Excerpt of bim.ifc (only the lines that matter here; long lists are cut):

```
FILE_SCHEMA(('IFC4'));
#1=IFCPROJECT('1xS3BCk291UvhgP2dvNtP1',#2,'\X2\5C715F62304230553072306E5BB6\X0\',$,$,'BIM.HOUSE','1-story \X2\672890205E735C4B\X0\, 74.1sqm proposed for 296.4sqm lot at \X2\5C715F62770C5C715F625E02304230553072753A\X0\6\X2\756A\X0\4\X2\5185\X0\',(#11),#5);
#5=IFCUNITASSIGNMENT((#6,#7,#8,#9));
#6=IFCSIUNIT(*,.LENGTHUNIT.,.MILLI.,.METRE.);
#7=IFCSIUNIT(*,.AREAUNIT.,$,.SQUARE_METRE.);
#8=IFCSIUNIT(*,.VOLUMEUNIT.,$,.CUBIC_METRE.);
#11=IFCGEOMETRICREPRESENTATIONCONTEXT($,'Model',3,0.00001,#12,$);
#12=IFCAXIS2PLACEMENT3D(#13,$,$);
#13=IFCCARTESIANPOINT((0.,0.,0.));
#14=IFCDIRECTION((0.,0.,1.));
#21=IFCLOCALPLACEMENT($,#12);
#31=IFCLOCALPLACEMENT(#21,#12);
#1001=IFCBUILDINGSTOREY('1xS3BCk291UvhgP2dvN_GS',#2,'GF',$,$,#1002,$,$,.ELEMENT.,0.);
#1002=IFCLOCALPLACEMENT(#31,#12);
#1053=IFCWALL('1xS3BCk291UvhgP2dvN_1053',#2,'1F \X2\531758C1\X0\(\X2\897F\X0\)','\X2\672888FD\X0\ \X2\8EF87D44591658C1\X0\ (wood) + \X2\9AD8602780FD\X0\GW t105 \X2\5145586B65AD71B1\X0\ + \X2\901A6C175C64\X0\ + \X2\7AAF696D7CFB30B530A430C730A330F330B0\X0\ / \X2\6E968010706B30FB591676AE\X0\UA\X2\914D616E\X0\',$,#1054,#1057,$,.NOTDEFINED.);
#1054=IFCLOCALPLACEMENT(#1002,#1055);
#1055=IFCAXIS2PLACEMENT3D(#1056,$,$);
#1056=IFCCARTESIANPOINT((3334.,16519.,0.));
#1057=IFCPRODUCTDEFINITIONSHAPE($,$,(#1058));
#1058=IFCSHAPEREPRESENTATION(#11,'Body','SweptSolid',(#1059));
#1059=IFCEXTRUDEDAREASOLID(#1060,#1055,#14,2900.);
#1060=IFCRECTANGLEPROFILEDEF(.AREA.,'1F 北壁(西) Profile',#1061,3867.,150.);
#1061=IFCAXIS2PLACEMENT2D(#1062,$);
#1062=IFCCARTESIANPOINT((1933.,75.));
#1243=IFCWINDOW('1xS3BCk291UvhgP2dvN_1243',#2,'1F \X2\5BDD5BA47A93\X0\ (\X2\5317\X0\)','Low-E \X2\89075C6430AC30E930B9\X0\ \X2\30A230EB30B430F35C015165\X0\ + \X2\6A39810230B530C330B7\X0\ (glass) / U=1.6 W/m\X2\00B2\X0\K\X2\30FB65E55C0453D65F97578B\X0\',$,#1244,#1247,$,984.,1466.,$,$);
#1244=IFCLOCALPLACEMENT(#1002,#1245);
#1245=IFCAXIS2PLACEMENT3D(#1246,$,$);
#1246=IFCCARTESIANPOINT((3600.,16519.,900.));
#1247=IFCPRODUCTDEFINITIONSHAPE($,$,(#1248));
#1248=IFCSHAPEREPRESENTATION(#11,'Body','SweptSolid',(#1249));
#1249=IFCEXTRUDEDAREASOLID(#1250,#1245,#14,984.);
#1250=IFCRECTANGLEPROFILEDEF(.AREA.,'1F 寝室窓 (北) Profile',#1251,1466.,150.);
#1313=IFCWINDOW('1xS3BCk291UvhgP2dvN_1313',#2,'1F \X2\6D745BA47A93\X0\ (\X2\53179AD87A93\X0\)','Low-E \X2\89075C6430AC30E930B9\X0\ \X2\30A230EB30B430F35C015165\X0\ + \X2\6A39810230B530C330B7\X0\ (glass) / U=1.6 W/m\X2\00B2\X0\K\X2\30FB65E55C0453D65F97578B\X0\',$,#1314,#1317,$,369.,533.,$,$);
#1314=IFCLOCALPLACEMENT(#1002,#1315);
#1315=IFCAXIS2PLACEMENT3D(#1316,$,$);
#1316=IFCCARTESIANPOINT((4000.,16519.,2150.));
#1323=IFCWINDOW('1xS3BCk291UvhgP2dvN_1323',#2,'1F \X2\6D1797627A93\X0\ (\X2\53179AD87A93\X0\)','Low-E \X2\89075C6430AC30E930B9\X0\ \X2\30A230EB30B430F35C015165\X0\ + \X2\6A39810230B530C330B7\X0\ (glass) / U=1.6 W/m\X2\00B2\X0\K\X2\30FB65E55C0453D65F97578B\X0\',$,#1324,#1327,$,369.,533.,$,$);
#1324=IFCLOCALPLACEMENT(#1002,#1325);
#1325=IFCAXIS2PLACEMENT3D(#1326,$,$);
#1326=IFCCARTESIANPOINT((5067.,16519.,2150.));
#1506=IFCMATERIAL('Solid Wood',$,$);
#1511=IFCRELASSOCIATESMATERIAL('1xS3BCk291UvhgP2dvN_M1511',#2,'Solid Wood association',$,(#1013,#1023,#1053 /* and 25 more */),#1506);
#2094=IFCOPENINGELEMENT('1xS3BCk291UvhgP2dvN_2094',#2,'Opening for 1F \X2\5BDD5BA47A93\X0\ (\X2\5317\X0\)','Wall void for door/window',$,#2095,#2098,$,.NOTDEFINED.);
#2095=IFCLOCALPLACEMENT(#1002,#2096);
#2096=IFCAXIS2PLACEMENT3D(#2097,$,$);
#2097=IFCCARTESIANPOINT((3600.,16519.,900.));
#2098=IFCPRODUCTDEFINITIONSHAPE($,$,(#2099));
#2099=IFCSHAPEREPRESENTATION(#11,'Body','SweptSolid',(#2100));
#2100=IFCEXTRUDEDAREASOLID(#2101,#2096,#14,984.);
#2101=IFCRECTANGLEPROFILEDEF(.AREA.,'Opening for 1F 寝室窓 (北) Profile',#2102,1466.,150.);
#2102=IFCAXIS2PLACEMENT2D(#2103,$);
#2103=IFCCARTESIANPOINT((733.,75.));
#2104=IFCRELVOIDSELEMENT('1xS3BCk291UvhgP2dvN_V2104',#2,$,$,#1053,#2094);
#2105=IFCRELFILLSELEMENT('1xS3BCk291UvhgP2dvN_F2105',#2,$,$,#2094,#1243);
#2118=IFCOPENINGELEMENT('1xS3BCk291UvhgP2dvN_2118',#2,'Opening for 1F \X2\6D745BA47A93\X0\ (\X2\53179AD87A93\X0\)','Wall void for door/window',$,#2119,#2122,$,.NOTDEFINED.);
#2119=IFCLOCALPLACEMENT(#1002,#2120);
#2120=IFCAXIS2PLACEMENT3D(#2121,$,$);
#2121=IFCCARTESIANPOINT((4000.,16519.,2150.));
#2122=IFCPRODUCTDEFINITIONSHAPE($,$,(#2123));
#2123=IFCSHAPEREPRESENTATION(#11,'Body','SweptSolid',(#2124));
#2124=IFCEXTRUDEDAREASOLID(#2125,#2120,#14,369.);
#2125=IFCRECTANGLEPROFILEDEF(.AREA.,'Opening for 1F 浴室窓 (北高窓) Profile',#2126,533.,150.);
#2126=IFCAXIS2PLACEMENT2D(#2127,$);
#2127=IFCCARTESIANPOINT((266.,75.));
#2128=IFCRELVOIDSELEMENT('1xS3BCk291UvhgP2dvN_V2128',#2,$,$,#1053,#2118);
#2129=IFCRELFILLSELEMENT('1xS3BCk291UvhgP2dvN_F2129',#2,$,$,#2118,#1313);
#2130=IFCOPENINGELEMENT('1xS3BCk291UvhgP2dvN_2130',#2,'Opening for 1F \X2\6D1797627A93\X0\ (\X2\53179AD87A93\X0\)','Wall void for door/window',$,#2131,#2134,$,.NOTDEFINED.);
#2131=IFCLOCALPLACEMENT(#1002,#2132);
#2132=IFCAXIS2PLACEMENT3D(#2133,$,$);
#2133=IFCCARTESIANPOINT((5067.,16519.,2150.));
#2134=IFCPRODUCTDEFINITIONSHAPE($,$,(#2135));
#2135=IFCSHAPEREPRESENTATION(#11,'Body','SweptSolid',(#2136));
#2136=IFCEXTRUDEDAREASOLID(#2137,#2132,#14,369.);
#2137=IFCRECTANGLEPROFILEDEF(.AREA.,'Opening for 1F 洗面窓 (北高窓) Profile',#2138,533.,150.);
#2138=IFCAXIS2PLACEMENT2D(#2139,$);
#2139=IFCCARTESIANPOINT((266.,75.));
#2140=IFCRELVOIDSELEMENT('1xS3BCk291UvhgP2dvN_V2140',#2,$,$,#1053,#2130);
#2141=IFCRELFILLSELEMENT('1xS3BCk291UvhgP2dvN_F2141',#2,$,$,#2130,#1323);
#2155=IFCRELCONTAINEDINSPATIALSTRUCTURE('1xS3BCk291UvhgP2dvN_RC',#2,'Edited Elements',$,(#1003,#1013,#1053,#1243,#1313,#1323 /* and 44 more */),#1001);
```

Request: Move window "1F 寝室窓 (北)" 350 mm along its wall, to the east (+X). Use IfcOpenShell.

```python
import ifcopenshell
import ifcopenshell.api.geometry
import ifcopenshell.util.placement

model = ifcopenshell.open("bim.ifc")

window = model.by_guid("1xS3BCk291UvhgP2dvN_1243")
opening = window.FillsVoids[0].RelatingOpeningElement
wall = opening.VoidsElements[0].RelatingBuildingElement

wall_matrix = ifcopenshell.util.placement.get_local_placement(wall.ObjectPlacement)
shift = wall_matrix[:3, 0] * 350.0
before = ifcopenshell.util.placement.get_local_placement(window.ObjectPlacement)[:3, 3].copy()

# The window is not placed relative to its opening, so move both.
for product in (opening, window):
    matrix = ifcopenshell.util.placement.get_local_placement(product.ObjectPlacement)
    matrix[:3, 3] += shift
    ifcopenshell.api.geometry.edit_object_placement(model, product=product, matrix=matrix, is_si=False)

after = ifcopenshell.util.placement.get_local_placement(window.ObjectPlacement)[:3, 3]
print("window moved by", (after - before).round(3) + 0.0)

model.write("bim_v2.ifc")
```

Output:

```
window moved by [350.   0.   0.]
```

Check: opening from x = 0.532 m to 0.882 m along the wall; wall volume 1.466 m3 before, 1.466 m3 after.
